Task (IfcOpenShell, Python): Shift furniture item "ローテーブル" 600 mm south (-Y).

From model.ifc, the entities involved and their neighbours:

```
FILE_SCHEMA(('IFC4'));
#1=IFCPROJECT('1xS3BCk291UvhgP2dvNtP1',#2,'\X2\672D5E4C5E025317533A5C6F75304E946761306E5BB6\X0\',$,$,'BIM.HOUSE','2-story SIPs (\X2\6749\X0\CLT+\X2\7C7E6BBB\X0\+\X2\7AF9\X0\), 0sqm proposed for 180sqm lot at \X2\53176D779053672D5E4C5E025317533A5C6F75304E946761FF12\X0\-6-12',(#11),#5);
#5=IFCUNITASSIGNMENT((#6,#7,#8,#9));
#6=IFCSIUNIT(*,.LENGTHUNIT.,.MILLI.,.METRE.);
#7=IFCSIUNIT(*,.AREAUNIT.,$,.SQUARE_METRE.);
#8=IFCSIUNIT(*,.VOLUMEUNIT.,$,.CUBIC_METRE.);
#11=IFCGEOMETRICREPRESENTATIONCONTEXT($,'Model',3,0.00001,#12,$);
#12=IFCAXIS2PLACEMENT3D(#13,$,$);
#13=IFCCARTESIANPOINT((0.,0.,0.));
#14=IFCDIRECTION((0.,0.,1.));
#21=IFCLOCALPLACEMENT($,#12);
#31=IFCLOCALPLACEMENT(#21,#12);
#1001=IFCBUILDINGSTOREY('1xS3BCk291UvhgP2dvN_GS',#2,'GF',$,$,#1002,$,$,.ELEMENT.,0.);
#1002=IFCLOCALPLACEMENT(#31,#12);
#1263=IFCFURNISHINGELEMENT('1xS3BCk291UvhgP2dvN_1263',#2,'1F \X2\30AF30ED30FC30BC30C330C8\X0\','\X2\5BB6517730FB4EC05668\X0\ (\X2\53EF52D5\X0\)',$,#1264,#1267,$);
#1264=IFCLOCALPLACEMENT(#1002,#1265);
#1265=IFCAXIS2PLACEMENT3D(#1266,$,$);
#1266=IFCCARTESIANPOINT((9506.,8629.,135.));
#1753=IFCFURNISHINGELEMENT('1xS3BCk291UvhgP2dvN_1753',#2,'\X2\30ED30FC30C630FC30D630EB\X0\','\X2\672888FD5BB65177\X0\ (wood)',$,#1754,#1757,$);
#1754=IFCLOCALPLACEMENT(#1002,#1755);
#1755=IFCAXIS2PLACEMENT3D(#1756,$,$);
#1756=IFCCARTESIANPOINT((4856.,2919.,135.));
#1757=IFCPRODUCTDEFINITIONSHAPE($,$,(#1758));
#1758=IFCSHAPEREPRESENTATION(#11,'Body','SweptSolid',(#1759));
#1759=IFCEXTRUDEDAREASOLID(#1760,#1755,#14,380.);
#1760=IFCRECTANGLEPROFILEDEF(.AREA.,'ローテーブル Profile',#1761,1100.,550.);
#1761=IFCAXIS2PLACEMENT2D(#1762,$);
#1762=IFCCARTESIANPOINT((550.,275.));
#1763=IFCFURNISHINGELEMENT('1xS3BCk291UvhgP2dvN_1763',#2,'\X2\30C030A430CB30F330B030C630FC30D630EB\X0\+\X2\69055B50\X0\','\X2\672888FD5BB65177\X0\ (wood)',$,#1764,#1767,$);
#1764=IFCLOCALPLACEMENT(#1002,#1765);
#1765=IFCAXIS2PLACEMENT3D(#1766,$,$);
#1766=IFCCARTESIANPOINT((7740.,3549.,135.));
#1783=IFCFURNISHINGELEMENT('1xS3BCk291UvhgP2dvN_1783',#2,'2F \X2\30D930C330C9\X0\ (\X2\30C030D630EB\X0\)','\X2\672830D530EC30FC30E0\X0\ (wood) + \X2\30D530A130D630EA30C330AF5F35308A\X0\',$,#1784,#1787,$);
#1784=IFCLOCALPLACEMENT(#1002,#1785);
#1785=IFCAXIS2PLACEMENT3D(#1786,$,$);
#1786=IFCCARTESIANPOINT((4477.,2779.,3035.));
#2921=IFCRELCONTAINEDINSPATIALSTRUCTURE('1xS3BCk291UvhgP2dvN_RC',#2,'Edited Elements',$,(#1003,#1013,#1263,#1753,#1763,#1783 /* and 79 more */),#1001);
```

```python
import ifcopenshell
import ifcopenshell.api.geometry
import ifcopenshell.util.placement

model = ifcopenshell.open("model.ifc")

item = model.by_guid("1xS3BCk291UvhgP2dvN_1753")
matrix = ifcopenshell.util.placement.get_local_placement(item.ObjectPlacement)
matrix[1, 3] -= 600.0
ifcopenshell.api.geometry.edit_object_placement(model, product=item, matrix=matrix, is_si=False)

print(ifcopenshell.util.placement.get_local_placement(item.ObjectPlacement).round(3) + 0.0)

model.write("model_rev.ifc")
```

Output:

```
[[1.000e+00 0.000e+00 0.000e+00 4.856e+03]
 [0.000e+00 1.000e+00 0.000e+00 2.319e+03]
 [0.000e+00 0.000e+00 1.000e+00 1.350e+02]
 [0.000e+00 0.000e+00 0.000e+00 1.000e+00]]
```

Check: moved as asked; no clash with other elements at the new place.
